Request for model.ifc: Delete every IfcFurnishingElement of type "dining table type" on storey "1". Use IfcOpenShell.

First a look at what the model holds.

```python
import ifcopenshell
import ifcopenshell.util.element

model = ifcopenshell.open("model.ifc")
print(model.schema)
storey = next(s for s in model.by_type("IfcBuildingStorey") if s.Name == "1")
furniture = [e for e in ifcopenshell.util.element.get_decomposition(storey) if e.is_a("IfcFurnishingElement")]
seen = {}
for e in furniture:
    element_type = ifcopenshell.util.element.get_type(e)
    name = element_type.Name if element_type not in (None, e) else None
    seen[name] = seen.get(name, 0) + 1
for name, count in sorted(seen.items(), key=str):
    print(count, "x", name)
```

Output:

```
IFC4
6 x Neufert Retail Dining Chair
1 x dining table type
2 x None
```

```python
import ifcopenshell
import ifcopenshell.api.root
import ifcopenshell.util.element

model = ifcopenshell.open("model.ifc")

storey = next(s for s in model.by_type("IfcBuildingStorey") if s.Name == "1")
furniture = [e for e in ifcopenshell.util.element.get_decomposition(storey) if e.is_a("IfcFurnishingElement")]
targets = [e for e in furniture if (t := ifcopenshell.util.element.get_type(e)) not in (None, e) and t.Name == "dining table type"]

for e in targets:
    ifcopenshell.api.root.remove_product(model, product=e)
print(len(targets), "removed")

model.write("model_rev.ifc")
```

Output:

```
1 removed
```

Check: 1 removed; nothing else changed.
